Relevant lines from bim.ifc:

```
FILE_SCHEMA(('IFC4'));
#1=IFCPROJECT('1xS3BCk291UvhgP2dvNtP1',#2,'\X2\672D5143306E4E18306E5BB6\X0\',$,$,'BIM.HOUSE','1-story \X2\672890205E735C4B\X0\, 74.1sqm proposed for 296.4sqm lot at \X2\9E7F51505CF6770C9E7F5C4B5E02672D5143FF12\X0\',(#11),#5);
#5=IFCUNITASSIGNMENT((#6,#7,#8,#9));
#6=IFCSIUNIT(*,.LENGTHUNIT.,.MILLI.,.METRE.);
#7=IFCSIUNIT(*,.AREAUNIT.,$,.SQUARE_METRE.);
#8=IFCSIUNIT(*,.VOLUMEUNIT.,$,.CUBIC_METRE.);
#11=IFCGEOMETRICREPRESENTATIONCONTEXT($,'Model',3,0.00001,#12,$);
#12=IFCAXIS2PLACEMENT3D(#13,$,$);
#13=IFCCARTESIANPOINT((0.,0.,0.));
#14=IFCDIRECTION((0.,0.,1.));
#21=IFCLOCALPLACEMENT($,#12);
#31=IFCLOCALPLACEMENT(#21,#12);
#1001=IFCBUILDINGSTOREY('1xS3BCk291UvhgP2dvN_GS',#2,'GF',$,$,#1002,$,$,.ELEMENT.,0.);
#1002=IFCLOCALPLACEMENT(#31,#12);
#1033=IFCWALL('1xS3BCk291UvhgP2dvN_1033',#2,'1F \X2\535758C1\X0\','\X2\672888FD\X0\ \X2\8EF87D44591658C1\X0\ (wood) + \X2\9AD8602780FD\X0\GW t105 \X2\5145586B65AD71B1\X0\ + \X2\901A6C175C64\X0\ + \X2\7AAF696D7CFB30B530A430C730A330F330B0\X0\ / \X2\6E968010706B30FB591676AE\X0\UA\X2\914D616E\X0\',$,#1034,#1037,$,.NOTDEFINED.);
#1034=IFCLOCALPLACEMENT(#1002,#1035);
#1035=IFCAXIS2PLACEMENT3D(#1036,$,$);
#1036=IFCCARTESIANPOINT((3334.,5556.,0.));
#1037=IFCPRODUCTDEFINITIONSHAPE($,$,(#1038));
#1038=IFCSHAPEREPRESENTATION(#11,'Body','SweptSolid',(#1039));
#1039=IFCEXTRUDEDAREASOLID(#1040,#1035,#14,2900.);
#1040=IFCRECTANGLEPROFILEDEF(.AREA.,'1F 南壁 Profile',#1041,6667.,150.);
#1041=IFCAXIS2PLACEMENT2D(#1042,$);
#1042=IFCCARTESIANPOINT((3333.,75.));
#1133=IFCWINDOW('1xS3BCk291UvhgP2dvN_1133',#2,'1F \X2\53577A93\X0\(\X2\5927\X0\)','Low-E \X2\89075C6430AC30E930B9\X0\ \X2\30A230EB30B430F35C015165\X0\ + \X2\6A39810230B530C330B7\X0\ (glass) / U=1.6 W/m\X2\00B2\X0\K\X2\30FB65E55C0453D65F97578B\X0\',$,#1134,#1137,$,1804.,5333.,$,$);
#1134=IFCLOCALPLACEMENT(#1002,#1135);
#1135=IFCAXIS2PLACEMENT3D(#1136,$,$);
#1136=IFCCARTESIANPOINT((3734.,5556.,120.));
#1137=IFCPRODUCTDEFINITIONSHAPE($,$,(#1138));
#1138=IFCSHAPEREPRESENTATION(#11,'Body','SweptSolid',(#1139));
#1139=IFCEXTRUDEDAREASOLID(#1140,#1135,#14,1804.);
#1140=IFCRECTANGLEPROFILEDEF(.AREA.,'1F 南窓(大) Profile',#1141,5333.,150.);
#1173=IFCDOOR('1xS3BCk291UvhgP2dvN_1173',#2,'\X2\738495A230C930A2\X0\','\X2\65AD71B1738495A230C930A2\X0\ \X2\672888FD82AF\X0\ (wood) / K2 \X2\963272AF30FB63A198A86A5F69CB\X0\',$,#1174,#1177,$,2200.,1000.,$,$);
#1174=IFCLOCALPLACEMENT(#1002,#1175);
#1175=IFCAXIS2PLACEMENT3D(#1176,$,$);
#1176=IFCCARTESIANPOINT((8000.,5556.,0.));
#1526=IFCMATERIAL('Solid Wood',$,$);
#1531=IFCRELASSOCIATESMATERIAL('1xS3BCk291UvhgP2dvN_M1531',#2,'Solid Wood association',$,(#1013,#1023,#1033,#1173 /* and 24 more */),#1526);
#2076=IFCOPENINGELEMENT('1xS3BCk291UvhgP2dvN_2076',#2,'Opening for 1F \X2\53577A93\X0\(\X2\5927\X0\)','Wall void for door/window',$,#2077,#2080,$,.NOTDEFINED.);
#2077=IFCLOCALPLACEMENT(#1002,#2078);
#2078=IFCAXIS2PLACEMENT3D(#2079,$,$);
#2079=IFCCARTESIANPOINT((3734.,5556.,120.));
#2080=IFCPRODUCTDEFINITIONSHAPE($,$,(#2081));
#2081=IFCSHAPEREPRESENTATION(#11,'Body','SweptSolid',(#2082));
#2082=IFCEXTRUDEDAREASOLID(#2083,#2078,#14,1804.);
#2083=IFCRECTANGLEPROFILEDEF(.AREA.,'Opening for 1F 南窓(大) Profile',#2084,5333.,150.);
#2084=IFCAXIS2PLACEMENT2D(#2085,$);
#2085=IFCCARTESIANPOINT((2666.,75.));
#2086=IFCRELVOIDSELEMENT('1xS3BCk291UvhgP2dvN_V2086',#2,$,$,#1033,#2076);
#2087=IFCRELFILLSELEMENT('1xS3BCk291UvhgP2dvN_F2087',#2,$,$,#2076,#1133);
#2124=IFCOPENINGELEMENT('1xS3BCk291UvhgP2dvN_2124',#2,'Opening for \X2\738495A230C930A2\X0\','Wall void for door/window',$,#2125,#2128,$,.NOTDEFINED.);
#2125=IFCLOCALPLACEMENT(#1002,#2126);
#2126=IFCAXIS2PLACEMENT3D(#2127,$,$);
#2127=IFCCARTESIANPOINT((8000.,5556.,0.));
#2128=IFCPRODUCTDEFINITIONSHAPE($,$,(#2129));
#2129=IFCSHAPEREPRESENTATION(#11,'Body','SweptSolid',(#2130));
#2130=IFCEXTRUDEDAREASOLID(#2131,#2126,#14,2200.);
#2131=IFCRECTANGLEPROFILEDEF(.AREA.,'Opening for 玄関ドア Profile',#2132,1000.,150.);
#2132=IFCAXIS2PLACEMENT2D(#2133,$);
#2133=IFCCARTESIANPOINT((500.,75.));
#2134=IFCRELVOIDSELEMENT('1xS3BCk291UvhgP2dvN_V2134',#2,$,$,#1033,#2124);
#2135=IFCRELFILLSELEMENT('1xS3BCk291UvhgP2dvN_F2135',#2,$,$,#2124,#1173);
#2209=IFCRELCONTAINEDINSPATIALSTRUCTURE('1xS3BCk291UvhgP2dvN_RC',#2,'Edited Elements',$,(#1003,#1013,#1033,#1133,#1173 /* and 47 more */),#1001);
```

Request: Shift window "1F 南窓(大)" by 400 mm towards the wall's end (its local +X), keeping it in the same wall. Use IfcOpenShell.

```python
import ifcopenshell
import ifcopenshell.api.geometry
import ifcopenshell.util.placement
import ifcopenshell.util.unit

model = ifcopenshell.open("bim.ifc")
unit_scale = ifcopenshell.util.unit.calculate_unit_scale(model)

window = model.by_guid("1xS3BCk291UvhgP2dvN_1133")
opening = window.FillsVoids[0].RelatingOpeningElement
wall = opening.VoidsElements[0].RelatingBuildingElement

wall_matrix = ifcopenshell.util.placement.get_local_placement(wall.ObjectPlacement)
shift = wall_matrix[:3, 0] * 0.4 / unit_scale
before = ifcopenshell.util.placement.get_local_placement(window.ObjectPlacement)[:3, 3].copy()

# The window is not placed relative to its opening, so move both.
for product in (opening, window):
    matrix = ifcopenshell.util.placement.get_local_placement(product.ObjectPlacement)
    matrix[:3, 3] += shift
    ifcopenshell.api.geometry.edit_object_placement(model, product=product, matrix=matrix, is_si=False)

after = ifcopenshell.util.placement.get_local_placement(window.ObjectPlacement)[:3, 3]
print("window moved by", (after - before).round(3) + 0.0)

model.write("bim_v2.ifc")
```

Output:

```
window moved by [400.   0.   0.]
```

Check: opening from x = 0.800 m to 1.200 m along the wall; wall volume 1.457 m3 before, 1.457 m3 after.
